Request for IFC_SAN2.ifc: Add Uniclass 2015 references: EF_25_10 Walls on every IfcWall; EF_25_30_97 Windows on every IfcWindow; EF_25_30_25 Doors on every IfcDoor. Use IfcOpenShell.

First a look at what the model holds.

```python
import ifcopenshell

model = ifcopenshell.open("IFC_SAN2.ifc")
print(model.schema)
print("classifications:", [c.Name for c in model.by_type("IfcClassification")])
for ifc_class in ("IfcDoor", "IfcRoof", "IfcStair", "IfcWall", "IfcWindow"):
    print(ifc_class, len(model.by_type(ifc_class)))
```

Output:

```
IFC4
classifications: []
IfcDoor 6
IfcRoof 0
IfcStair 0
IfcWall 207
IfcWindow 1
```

```python
import ifcopenshell
import ifcopenshell.api.classification

model = ifcopenshell.open("IFC_SAN2.ifc")

system = ifcopenshell.api.classification.add_classification(model, classification="Uniclass 2015")

codes = {
    "IfcWall": ("EF_25_10", "Walls"),
    "IfcWindow": ("EF_25_30_97", "Windows"),
    "IfcDoor": ("EF_25_30_25", "Doors"),
}
for ifc_class, (code, name) in codes.items():
    products = model.by_type(ifc_class)
    ifcopenshell.api.classification.add_reference(
        model, products=products, classification=system, identification=code, name=name
    )
    print(code, len(products))

model.write("IFC_SAN2_rev.ifc")
```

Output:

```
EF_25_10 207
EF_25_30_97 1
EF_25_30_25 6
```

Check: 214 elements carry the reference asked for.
